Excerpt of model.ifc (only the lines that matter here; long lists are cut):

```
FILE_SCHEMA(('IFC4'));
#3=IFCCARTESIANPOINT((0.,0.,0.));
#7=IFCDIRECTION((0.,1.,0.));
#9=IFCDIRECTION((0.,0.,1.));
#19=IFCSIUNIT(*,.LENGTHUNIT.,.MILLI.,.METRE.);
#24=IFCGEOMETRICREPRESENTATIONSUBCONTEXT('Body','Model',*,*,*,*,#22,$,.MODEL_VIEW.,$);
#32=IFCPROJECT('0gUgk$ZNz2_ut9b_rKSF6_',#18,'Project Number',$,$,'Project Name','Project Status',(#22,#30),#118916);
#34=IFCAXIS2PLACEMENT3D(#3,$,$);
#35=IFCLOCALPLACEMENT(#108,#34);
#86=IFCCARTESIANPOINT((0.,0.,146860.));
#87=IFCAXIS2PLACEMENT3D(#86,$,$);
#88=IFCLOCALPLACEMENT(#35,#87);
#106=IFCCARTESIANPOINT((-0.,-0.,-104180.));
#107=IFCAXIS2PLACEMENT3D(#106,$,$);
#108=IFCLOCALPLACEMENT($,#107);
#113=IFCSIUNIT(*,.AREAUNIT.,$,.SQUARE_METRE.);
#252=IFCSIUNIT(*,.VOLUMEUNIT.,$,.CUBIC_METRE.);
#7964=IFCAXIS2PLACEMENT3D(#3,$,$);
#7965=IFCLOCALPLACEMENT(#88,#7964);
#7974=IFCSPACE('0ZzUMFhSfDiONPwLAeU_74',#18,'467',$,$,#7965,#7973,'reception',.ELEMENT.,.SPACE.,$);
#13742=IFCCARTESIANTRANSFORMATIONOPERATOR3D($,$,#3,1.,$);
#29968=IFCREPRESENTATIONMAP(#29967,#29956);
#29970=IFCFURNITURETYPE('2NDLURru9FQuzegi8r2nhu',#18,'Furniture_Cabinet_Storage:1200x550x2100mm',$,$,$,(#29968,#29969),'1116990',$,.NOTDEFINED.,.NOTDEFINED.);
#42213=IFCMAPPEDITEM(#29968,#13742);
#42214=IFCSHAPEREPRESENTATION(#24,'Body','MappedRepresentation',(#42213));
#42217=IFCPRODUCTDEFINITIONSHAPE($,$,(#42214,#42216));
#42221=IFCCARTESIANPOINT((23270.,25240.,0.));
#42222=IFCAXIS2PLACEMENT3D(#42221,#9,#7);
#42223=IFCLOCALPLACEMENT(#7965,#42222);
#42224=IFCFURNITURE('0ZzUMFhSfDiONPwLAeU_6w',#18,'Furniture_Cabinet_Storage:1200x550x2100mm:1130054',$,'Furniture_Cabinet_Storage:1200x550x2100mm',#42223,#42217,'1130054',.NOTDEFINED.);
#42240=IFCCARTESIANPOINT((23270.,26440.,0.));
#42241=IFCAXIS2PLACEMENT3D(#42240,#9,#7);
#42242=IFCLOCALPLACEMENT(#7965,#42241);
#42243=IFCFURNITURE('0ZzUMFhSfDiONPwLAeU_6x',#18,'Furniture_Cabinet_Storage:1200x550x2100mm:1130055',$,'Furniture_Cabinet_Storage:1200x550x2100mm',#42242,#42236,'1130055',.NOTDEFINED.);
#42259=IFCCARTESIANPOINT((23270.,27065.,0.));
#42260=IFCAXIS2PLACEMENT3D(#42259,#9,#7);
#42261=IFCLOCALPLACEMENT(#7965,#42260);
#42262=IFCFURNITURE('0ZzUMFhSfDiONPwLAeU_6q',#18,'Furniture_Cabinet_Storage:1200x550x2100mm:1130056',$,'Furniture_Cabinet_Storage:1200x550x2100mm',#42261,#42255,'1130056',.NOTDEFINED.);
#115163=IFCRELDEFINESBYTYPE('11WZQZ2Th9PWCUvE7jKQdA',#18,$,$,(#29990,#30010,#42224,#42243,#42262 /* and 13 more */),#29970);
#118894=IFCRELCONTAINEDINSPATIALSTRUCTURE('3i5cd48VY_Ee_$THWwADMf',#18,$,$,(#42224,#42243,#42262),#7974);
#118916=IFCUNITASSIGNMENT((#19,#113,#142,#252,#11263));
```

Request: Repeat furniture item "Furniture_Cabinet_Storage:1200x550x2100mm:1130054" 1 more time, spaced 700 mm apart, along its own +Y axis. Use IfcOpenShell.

```python
import ifcopenshell
import ifcopenshell.api.geometry
import ifcopenshell.api.root
import ifcopenshell.util.element
import ifcopenshell.util.placement

model = ifcopenshell.open("model.ifc")


def reuse_history(source, copy):
    """copy_class also copies each property set's owner history, people and application; keep the originals."""
    for rel in copy.IsDefinedBy:
        if rel.is_a("IfcRelDefinesByProperties") and (history := rel.RelatingPropertyDefinition.OwnerHistory):
            rel.RelatingPropertyDefinition.OwnerHistory = source.OwnerHistory
            ifcopenshell.util.element.remove_deep2(model, history)


source = model.by_guid("0ZzUMFhSfDiONPwLAeU_6w")
base = ifcopenshell.util.placement.get_local_placement(source.ObjectPlacement)
step = base[:3, 1] * 700.0

for i in range(1, 2):
    copy = ifcopenshell.api.root.copy_class(model, product=source)
    copy.Representation = ifcopenshell.util.element.copy_deep(
        model, source.Representation, exclude=["IfcGeometricRepresentationContext", "IfcRepresentationMap"]
    )
    copy.Name = "Furniture_Cabinet_Storage:1200x550x2100mm"
    copy.Tag = None
    reuse_history(source, copy)
    matrix = base.copy()
    matrix[:3, 3] += i * step
    print("added at", matrix[:3, 3].round(3) + 0.0)
    ifcopenshell.api.geometry.edit_object_placement(model, product=copy, matrix=matrix, is_si=False)

model.write("model_rev.ifc")
```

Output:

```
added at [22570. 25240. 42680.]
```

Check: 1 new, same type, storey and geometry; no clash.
